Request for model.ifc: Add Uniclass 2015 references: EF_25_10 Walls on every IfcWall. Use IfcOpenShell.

First a look at what the model holds.

```python
import ifcopenshell

model = ifcopenshell.open("model.ifc")
print(model.schema)
print("classifications:", [c.Name for c in model.by_type("IfcClassification")])
for ifc_class in ("IfcDoor", "IfcRoof", "IfcStair", "IfcWall", "IfcWindow"):
    print(ifc_class, len(model.by_type(ifc_class)))
```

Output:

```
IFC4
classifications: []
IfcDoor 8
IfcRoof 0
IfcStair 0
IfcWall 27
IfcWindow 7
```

```python
import ifcopenshell
import ifcopenshell.api.classification

model = ifcopenshell.open("model.ifc")

system = ifcopenshell.api.classification.add_classification(model, classification="Uniclass 2015")

codes = {
    "IfcWall": ("EF_25_10", "Walls"),
}
for ifc_class, (code, name) in codes.items():
    products = model.by_type(ifc_class)
    ifcopenshell.api.classification.add_reference(
        model, products=products, classification=system, identification=code, name=name
    )
    print(code, len(products))

model.write("model_rev.ifc")
```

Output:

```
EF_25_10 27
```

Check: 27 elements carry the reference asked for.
